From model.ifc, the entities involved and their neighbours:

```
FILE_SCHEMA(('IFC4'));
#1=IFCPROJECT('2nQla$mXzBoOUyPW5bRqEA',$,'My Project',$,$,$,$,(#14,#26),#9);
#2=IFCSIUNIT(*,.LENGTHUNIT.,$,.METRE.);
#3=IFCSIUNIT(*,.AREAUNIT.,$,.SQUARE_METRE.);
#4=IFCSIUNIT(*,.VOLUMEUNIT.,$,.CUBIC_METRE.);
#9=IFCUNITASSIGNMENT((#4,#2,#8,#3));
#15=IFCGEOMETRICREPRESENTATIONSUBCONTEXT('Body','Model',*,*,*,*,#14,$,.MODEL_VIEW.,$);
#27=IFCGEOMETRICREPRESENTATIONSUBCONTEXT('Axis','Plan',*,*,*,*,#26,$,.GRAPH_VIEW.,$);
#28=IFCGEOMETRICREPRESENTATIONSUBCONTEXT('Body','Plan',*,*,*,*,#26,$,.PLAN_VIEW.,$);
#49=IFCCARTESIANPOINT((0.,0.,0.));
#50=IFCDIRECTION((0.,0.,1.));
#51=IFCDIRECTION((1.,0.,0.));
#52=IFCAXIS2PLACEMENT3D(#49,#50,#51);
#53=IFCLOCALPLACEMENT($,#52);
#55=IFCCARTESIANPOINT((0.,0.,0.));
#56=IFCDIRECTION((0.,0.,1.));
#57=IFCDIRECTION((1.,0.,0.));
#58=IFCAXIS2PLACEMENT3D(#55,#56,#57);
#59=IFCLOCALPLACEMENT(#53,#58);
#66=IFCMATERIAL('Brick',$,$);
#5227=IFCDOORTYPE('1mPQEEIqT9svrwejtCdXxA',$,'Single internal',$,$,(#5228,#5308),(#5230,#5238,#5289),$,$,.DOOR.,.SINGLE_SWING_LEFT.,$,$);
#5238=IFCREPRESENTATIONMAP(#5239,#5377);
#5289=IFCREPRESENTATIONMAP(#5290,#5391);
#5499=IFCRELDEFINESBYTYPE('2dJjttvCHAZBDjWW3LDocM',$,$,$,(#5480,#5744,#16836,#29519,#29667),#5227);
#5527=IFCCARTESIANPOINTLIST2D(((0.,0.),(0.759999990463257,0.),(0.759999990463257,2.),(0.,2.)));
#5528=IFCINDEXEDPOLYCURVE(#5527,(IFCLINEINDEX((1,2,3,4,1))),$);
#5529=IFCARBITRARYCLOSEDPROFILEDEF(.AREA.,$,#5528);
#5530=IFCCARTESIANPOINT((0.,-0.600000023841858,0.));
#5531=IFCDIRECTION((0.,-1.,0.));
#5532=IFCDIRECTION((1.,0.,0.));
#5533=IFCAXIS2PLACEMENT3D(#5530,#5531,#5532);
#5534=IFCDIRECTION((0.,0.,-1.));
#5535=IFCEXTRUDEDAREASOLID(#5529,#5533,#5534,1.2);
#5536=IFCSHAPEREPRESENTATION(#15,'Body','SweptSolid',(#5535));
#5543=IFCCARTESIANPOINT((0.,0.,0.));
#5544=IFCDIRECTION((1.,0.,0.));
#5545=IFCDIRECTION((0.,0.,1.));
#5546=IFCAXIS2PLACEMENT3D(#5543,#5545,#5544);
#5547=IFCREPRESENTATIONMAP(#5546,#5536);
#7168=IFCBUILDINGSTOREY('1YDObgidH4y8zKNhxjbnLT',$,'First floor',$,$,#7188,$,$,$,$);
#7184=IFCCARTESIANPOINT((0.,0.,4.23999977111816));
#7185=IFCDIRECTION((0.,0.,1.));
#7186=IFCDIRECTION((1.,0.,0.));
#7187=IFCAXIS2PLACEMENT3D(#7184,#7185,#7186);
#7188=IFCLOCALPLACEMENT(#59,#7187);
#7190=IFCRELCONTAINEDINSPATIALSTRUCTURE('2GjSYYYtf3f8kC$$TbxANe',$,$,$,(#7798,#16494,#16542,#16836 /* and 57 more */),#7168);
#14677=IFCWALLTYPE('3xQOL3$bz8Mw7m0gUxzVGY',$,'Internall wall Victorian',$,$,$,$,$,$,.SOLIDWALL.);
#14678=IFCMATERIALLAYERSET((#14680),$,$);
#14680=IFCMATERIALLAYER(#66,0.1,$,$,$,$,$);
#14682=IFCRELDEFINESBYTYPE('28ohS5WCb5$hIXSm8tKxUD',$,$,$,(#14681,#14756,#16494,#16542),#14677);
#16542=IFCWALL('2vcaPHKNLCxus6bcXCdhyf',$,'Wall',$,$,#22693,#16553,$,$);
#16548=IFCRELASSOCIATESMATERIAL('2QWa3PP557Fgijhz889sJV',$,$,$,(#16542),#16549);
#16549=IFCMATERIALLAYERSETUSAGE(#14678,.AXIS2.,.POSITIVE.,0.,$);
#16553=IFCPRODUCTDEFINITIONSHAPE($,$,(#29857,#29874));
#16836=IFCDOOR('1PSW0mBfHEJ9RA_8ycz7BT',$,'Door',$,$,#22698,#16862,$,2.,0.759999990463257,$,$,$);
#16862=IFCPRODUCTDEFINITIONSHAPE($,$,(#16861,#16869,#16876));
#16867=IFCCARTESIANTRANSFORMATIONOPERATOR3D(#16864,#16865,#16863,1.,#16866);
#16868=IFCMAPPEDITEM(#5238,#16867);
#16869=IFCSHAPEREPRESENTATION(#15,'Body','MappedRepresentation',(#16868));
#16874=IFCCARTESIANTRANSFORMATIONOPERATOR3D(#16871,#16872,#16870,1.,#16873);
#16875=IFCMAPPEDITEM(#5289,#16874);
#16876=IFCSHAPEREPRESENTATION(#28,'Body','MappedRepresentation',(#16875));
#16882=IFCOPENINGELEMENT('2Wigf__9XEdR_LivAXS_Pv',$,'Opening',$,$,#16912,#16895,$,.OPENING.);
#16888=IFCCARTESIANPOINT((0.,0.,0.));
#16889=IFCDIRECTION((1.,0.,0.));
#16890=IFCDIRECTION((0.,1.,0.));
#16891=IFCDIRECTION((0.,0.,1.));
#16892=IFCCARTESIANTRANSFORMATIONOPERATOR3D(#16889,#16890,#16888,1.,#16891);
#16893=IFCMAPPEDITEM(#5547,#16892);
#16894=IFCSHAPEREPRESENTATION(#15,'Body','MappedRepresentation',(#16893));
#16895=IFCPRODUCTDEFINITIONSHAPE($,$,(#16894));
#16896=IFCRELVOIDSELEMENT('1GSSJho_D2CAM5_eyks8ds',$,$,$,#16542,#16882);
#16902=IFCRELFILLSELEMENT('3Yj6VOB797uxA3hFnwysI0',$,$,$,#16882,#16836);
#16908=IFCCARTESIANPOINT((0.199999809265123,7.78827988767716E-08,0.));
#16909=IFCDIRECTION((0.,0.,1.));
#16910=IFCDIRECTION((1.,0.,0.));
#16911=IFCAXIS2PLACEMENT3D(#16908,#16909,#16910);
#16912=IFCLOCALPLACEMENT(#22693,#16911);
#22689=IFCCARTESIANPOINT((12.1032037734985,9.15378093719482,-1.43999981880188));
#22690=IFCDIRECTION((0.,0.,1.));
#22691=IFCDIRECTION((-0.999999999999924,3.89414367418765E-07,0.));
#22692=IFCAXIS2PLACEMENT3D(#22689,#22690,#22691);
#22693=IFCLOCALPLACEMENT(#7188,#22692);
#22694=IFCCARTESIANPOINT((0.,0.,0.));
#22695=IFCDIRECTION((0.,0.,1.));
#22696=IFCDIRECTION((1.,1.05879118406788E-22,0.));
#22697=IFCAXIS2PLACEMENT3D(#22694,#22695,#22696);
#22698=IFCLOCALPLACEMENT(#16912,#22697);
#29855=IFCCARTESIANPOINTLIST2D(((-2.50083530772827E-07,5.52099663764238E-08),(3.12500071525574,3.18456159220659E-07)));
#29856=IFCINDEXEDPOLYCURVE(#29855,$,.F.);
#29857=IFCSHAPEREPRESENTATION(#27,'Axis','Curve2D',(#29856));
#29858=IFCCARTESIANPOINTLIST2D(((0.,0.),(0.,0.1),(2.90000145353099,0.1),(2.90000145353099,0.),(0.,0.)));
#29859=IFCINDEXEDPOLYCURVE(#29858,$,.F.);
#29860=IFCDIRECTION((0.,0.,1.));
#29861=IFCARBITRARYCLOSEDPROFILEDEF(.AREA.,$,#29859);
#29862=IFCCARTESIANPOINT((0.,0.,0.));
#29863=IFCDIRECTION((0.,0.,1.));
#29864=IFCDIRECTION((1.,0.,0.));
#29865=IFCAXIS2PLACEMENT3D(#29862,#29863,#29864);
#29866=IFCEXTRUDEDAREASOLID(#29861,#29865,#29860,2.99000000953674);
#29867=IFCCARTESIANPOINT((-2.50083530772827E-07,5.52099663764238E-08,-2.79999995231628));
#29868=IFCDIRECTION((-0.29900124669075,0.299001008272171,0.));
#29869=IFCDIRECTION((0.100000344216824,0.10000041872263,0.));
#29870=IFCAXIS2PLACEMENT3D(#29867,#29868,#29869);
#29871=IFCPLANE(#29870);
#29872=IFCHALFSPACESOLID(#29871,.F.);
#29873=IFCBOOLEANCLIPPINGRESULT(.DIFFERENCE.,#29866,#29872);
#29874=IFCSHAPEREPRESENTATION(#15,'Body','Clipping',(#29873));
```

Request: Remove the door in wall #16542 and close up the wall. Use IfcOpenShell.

```python
import ifcopenshell
import ifcopenshell.api.feature
import ifcopenshell.api.root
import ifcopenshell.geom
import ifcopenshell.util.shape

model = ifcopenshell.open("model.ifc")
settings = ifcopenshell.geom.settings()


def volume(element):
    """Net volume in cubic metres, openings subtracted."""
    shape = ifcopenshell.geom.create_shape(settings, element)
    return ifcopenshell.util.shape.get_volume(shape.geometry)


door = model.by_guid("1PSW0mBfHEJ9RA_8ycz7BT")
opening = door.FillsVoids[0].RelatingOpeningElement
wall = opening.VoidsElements[0].RelatingBuildingElement
before = volume(wall)

ifcopenshell.api.root.remove_product(model, product=door)
ifcopenshell.api.feature.remove_feature(model, feature=opening)

after = volume(wall)

print(f"wall volume {before:.3f} -> {after:.3f} m3")

model.write("model_updated.ifc")
```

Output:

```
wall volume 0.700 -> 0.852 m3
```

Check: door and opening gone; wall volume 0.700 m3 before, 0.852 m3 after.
